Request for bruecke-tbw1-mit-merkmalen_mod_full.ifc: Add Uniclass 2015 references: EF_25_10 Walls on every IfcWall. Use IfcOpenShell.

First a look at what the model holds.

```python
import ifcopenshell

model = ifcopenshell.open("bruecke-tbw1-mit-merkmalen_mod_full.ifc")
print(model.schema)
print("classifications:", [c.Name for c in model.by_type("IfcClassification")])
for ifc_class in ("IfcDoor", "IfcRoof", "IfcStair", "IfcWall", "IfcWindow"):
    print(ifc_class, len(model.by_type(ifc_class)))
```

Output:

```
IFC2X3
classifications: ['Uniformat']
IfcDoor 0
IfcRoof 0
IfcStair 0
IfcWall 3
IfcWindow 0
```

```python
import ifcopenshell
import ifcopenshell.api.classification

model = ifcopenshell.open("bruecke-tbw1-mit-merkmalen_mod_full.ifc")

# IFC2X3 requires Source and Edition and has no link from the project to the system.
system = model.create_entity("IfcClassification", Source="NBS", Edition="2015", Name="Uniclass 2015")

codes = {
    "IfcWall": ("EF_25_10", "Walls"),
}
for ifc_class, (code, name) in codes.items():
    products = model.by_type(ifc_class)
    ifcopenshell.api.classification.add_reference(
        model, products=products, classification=system, identification=code, name=name
    )
    print(code, len(products))

model.write("bruecke-tbw1-mit-merkmalen_mod_full_v2.ifc")
```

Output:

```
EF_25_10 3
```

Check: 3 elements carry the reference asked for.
